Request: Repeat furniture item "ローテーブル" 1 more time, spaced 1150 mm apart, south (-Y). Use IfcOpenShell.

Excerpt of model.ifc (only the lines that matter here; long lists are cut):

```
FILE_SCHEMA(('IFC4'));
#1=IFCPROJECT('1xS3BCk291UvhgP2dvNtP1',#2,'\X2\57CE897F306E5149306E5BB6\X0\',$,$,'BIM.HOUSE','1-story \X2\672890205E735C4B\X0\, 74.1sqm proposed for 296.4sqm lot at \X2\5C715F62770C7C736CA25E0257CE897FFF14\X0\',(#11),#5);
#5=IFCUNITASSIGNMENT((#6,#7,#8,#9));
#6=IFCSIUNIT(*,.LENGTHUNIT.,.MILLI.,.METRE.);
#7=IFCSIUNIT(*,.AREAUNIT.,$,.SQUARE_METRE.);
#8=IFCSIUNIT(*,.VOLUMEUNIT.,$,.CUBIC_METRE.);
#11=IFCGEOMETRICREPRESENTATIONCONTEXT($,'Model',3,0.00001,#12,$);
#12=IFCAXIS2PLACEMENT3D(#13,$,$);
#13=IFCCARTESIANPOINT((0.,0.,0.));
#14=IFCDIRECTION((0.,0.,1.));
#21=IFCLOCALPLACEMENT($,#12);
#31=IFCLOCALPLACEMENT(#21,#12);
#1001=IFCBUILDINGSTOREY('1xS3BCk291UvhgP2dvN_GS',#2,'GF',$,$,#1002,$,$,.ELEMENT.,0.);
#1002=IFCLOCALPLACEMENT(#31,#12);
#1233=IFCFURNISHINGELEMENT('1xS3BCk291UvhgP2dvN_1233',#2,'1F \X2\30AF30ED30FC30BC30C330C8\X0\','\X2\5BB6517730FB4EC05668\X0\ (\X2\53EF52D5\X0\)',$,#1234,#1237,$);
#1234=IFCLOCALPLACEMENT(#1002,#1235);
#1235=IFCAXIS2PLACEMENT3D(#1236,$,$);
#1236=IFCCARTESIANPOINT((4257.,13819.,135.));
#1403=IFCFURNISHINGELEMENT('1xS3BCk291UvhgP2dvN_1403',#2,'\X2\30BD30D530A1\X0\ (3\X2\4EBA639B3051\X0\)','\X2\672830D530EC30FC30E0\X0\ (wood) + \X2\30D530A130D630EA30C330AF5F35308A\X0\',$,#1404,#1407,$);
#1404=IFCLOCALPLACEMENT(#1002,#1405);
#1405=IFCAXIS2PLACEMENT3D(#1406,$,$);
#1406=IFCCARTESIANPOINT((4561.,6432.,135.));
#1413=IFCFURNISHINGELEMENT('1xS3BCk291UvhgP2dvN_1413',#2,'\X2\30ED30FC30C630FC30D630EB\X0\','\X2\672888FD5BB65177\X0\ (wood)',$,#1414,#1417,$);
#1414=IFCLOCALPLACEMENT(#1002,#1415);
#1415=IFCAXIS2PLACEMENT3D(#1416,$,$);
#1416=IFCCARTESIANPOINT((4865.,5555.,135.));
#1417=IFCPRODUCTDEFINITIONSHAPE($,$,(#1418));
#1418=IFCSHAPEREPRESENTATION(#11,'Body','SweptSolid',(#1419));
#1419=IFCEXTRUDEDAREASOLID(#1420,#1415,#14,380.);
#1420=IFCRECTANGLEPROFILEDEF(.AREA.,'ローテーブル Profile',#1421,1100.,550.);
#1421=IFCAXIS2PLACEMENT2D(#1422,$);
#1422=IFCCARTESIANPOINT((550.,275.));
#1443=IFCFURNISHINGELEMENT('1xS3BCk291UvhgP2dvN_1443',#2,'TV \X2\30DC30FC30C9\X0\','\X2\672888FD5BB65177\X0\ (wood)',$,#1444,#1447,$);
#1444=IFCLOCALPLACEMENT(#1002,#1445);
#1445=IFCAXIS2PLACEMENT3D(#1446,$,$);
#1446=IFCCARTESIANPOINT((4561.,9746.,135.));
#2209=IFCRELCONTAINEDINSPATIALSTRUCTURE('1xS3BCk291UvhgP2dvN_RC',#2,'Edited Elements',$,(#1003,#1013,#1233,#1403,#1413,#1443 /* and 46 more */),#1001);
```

```python
import numpy as np
import ifcopenshell
import ifcopenshell.api.geometry
import ifcopenshell.api.root
import ifcopenshell.util.element
import ifcopenshell.util.placement

model = ifcopenshell.open("model.ifc")


def reuse_history(source, copy):
    """copy_class also copies each property set's owner history, people and application; keep the originals."""
    for rel in copy.IsDefinedBy:
        if rel.is_a("IfcRelDefinesByProperties") and (history := rel.RelatingPropertyDefinition.OwnerHistory):
            rel.RelatingPropertyDefinition.OwnerHistory = source.OwnerHistory
            ifcopenshell.util.element.remove_deep2(model, history)


source = model.by_id(1413)
base = ifcopenshell.util.placement.get_local_placement(source.ObjectPlacement)
step = np.array([0.0, -1.0, 0.0]) * 1150.0

for i in range(1, 2):
    copy = ifcopenshell.api.root.copy_class(model, product=source)
    copy.Representation = ifcopenshell.util.element.copy_deep(
        model, source.Representation, exclude=["IfcGeometricRepresentationContext", "IfcRepresentationMap"]
    )
    reuse_history(source, copy)
    matrix = base.copy()
    matrix[:3, 3] += i * step
    print("added at", matrix[:3, 3].round(3) + 0.0)
    ifcopenshell.api.geometry.edit_object_placement(model, product=copy, matrix=matrix, is_si=False)

model.write("model_updated.ifc")
```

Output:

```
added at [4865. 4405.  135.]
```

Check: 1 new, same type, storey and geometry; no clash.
